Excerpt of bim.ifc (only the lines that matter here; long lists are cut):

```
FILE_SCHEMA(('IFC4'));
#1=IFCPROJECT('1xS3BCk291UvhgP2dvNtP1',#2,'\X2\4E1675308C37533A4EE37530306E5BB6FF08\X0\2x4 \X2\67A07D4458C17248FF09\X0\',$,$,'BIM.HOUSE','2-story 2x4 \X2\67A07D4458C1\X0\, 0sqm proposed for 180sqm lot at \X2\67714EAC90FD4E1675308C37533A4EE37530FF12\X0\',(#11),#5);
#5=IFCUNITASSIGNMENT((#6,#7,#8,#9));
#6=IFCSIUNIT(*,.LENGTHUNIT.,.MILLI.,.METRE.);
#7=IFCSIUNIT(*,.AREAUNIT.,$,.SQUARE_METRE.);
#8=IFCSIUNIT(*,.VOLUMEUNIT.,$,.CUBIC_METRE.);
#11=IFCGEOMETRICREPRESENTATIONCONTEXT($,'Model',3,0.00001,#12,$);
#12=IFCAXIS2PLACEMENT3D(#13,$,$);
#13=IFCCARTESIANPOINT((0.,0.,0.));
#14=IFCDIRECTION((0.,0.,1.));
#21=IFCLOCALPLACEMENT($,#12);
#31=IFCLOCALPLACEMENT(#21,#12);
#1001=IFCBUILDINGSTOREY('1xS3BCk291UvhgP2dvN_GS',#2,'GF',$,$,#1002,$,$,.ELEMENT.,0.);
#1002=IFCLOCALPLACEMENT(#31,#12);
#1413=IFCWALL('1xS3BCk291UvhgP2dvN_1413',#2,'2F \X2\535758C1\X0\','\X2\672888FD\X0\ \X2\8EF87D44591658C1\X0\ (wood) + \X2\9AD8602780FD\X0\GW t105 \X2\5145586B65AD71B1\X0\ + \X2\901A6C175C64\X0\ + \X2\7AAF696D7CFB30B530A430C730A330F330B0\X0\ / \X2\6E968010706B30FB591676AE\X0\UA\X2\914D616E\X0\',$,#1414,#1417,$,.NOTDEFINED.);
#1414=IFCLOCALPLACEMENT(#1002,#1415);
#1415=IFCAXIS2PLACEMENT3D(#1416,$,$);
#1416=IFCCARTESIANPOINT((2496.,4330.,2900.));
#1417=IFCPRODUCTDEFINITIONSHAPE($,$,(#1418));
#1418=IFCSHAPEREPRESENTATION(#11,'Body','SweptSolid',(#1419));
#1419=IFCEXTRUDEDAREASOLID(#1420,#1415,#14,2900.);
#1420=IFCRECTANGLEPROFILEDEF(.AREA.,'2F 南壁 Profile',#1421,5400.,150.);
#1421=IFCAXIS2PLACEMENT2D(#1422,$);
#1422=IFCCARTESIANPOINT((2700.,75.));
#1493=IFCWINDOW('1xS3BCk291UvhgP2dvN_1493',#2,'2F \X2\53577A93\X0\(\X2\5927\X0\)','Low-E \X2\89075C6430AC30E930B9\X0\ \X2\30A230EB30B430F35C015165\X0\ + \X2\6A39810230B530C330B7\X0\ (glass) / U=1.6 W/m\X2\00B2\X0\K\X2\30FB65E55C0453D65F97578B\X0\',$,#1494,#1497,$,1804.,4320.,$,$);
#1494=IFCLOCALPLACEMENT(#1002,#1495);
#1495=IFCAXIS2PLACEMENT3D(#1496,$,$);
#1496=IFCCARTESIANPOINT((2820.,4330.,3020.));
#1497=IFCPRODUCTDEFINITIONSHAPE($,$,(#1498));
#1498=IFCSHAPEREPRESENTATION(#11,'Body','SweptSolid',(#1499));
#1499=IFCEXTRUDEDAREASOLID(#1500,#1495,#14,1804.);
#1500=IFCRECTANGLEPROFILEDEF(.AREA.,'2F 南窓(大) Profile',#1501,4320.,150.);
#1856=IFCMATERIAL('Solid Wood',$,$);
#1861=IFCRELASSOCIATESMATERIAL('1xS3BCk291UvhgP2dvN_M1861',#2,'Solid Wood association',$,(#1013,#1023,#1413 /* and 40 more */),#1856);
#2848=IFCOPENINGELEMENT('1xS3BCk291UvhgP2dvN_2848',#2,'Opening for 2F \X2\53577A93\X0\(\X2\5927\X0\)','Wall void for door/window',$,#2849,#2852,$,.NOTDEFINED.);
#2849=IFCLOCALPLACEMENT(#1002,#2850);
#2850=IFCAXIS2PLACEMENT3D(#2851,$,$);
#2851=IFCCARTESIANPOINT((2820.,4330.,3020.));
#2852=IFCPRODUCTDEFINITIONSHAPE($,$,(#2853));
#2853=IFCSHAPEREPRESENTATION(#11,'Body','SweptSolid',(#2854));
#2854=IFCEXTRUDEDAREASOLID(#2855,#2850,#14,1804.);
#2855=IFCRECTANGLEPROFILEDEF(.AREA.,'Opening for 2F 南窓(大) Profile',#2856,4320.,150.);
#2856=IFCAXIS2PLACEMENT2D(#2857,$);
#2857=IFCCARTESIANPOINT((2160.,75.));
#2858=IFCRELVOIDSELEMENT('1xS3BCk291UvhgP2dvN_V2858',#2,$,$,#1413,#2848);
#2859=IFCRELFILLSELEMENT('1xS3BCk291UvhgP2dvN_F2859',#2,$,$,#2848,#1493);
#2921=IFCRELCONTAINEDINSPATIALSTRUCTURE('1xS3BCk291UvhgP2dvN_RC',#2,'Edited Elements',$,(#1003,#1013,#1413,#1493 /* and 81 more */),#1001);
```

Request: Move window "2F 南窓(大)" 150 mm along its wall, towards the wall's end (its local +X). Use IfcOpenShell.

```python
import ifcopenshell
import ifcopenshell.api.geometry
import ifcopenshell.util.placement
import ifcopenshell.util.unit

model = ifcopenshell.open("bim.ifc")
unit_scale = ifcopenshell.util.unit.calculate_unit_scale(model)

window = model.by_guid("1xS3BCk291UvhgP2dvN_1493")
opening = window.FillsVoids[0].RelatingOpeningElement
wall = opening.VoidsElements[0].RelatingBuildingElement

wall_matrix = ifcopenshell.util.placement.get_local_placement(wall.ObjectPlacement)
shift = wall_matrix[:3, 0] * 0.15 / unit_scale
before = ifcopenshell.util.placement.get_local_placement(window.ObjectPlacement)[:3, 3].copy()

# The window is not placed relative to its opening, so move both.
for product in (opening, window):
    matrix = ifcopenshell.util.placement.get_local_placement(product.ObjectPlacement)
    matrix[:3, 3] += shift
    ifcopenshell.api.geometry.edit_object_placement(model, product=product, matrix=matrix, is_si=False)

after = ifcopenshell.util.placement.get_local_placement(window.ObjectPlacement)[:3, 3]
print("window moved by", (after - before).round(3) + 0.0)

model.write("bim-out.ifc")
```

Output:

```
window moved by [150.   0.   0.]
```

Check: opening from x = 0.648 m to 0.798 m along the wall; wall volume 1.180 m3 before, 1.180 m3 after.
